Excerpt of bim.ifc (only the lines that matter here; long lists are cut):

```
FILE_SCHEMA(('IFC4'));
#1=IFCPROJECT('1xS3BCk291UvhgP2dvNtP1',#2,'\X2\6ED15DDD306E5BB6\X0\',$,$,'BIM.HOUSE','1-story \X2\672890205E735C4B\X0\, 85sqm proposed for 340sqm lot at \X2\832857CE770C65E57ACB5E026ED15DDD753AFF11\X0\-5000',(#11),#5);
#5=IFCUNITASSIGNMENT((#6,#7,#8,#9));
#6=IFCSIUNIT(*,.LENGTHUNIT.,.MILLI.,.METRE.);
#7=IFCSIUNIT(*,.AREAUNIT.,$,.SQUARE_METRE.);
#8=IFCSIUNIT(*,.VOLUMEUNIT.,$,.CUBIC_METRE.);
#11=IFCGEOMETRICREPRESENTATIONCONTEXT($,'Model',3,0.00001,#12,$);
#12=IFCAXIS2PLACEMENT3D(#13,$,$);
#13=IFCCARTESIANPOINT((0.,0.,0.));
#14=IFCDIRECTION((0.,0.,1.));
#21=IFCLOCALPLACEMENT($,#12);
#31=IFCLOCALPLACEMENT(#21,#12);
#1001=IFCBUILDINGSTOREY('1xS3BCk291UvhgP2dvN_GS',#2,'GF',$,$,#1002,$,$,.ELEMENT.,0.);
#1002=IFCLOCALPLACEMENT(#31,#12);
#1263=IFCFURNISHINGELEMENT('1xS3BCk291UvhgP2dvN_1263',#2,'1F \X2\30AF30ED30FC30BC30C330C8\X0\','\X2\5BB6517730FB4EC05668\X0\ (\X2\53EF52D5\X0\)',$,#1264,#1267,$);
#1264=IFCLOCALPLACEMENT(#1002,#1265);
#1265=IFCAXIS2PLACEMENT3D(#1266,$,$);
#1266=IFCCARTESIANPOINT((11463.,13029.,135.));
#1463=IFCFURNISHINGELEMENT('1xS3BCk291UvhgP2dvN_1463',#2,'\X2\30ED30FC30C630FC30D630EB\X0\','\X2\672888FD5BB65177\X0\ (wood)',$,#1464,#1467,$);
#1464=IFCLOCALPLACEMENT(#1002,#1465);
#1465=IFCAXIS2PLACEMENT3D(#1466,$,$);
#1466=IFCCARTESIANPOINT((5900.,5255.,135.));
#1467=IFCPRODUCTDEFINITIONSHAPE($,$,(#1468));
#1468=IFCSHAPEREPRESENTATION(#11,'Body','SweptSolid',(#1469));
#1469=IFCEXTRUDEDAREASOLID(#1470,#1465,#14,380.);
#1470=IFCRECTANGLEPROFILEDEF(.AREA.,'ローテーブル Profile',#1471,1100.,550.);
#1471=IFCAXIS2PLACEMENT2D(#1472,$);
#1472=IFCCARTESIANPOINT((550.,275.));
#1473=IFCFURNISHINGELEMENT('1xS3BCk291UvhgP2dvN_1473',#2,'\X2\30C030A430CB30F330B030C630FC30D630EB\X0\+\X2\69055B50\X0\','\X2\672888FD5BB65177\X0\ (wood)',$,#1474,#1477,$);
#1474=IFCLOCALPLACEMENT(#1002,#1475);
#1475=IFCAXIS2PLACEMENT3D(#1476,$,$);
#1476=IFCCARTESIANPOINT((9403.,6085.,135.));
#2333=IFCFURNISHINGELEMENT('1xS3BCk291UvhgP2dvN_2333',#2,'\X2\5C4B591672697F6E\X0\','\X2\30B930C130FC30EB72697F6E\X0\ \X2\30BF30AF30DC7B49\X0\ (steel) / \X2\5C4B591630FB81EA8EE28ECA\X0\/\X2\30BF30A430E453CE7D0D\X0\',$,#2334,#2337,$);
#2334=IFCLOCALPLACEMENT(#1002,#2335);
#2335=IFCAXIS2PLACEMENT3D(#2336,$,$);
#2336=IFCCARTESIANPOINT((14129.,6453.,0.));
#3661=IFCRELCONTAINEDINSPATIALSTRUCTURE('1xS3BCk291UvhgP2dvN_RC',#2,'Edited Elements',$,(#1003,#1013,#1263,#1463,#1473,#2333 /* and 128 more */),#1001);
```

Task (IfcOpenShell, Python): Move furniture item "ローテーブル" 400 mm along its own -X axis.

```python
import ifcopenshell
import ifcopenshell.api.geometry
import ifcopenshell.util.placement
import ifcopenshell.util.unit

model = ifcopenshell.open("bim.ifc")
unit_scale = ifcopenshell.util.unit.calculate_unit_scale(model)

item = model.by_guid("1xS3BCk291UvhgP2dvN_1463")
matrix = ifcopenshell.util.placement.get_local_placement(item.ObjectPlacement)
matrix[:3, 3] -= matrix[:3, 0] * 0.4 / unit_scale
ifcopenshell.api.geometry.edit_object_placement(model, product=item, matrix=matrix, is_si=False)

print(ifcopenshell.util.placement.get_local_placement(item.ObjectPlacement).round(3) + 0.0)

model.write("bim-out.ifc")
```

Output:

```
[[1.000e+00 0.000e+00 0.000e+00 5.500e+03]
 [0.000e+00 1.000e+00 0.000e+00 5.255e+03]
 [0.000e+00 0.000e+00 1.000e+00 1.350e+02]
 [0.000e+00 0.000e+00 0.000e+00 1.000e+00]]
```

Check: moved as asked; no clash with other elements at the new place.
